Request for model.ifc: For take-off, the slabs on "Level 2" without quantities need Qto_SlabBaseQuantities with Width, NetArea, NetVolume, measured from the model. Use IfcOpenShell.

First a look at what the model holds.

```python
import ifcopenshell
import ifcopenshell.util.element
import ifcopenshell.util.unit

model = ifcopenshell.open("model.ifc")
print(model.schema)
for unit_type in ("LENGTHUNIT", "AREAUNIT", "VOLUMEUNIT"):
    print(unit_type, ifcopenshell.util.unit.calculate_unit_scale(model, unit_type))
storey = next(s for s in model.by_type("IfcBuildingStorey") if s.Name == "Level 2")
slabs = [e for e in ifcopenshell.util.element.get_decomposition(storey) if e.is_a("IfcSlab")]
for e in sorted(slabs, key=lambda e: e.id()):
    print(e.id(), e.is_a(), e.Name, list(ifcopenshell.util.element.get_psets(e, qtos_only=True)), sep=" | ")
```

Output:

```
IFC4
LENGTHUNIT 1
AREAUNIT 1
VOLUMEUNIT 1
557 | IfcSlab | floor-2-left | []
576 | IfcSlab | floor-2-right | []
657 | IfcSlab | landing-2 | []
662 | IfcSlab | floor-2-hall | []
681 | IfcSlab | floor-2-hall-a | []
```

```python
import ifcopenshell
import ifcopenshell.api.pset
import ifcopenshell.geom
import ifcopenshell.util.element
import ifcopenshell.util.shape
import ifcopenshell.util.unit

model = ifcopenshell.open("model.ifc")
unit_scale = ifcopenshell.util.unit.calculate_unit_scale(model)
area_scale = ifcopenshell.util.unit.calculate_unit_scale(model, "AREAUNIT")
volume_scale = ifcopenshell.util.unit.calculate_unit_scale(model, "VOLUMEUNIT")
settings = ifcopenshell.geom.settings()

storey = next(s for s in model.by_type("IfcBuildingStorey") if s.Name == "Level 2")
slabs = [e for e in ifcopenshell.util.element.get_decomposition(storey) if e.is_a("IfcSlab")]

for e in sorted(slabs, key=lambda e: e.id()):
    if ifcopenshell.util.element.get_psets(e, qtos_only=True, should_inherit=False):
        continue
    # Geometry comes back in metres, in the element's own axes.
    shape = ifcopenshell.geom.create_shape(settings, e)
    values = {
        "Width": ifcopenshell.util.shape.get_z(shape.geometry) / unit_scale,
        "NetArea": ifcopenshell.util.shape.get_footprint_area(shape.geometry) / area_scale,
        "NetVolume": ifcopenshell.util.shape.get_volume(shape.geometry) / volume_scale,
    }
    qto = ifcopenshell.api.pset.add_qto(model, product=e, name="Qto_SlabBaseQuantities")
    ifcopenshell.api.pset.edit_qto(model, qto=qto, properties=values)
    print(e.id(), {k: round(v, 3) for k, v in values.items()})

model.write("model_edited.ifc")
```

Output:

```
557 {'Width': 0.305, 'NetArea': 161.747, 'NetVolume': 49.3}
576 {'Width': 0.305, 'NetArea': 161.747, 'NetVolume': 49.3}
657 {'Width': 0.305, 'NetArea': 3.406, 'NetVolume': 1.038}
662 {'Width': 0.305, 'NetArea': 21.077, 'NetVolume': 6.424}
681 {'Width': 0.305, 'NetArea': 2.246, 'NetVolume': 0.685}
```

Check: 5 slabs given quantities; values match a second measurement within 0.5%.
